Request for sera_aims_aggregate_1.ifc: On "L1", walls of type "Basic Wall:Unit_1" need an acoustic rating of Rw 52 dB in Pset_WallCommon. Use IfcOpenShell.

First a look at what the model holds.

```python
import ifcopenshell
import ifcopenshell.util.element

model = ifcopenshell.open("sera_aims_aggregate_1.ifc")
print(model.schema)
storey = next(s for s in model.by_type("IfcBuildingStorey") if s.Name == "L1")
walls = [e for e in ifcopenshell.util.element.get_decomposition(storey) if e.is_a("IfcWall")]
seen = {}
for e in walls:
    element_type = ifcopenshell.util.element.get_type(e)
    key = (element_type.Name if element_type != e and element_type else None, ifcopenshell.util.element.get_pset(e, "Pset_WallCommon", "AcousticRating"))
    seen[key] = seen.get(key, 0) + 1
for (name, value), count in sorted(seen.items(), key=str):
    print(count, "x", name, "|", value)
```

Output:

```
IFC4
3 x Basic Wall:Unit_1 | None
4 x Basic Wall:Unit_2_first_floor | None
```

```python
import ifcopenshell
import ifcopenshell.api.pset
import ifcopenshell.util.element

model = ifcopenshell.open("sera_aims_aggregate_1.ifc")

storey = next(s for s in model.by_type("IfcBuildingStorey") if s.Name == "L1")
walls = [e for e in ifcopenshell.util.element.get_decomposition(storey) if e.is_a("IfcWall")]

count = 0
for e in walls:
    element_type = ifcopenshell.util.element.get_type(e)
    if element_type in (None, e) or element_type.Name != "Basic Wall:Unit_1":
        continue
    # add_pset returns the element's existing set when there is one.
    pset = ifcopenshell.api.pset.add_pset(model, product=e, name="Pset_WallCommon")
    ifcopenshell.api.pset.edit_pset(model, pset=pset, properties={"AcousticRating": "Rw 52 dB"})
    count += 1

print(count, "walls updated")

model.write("sera_aims_aggregate_1_v2.ifc")
```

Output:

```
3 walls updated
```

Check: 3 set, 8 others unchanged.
